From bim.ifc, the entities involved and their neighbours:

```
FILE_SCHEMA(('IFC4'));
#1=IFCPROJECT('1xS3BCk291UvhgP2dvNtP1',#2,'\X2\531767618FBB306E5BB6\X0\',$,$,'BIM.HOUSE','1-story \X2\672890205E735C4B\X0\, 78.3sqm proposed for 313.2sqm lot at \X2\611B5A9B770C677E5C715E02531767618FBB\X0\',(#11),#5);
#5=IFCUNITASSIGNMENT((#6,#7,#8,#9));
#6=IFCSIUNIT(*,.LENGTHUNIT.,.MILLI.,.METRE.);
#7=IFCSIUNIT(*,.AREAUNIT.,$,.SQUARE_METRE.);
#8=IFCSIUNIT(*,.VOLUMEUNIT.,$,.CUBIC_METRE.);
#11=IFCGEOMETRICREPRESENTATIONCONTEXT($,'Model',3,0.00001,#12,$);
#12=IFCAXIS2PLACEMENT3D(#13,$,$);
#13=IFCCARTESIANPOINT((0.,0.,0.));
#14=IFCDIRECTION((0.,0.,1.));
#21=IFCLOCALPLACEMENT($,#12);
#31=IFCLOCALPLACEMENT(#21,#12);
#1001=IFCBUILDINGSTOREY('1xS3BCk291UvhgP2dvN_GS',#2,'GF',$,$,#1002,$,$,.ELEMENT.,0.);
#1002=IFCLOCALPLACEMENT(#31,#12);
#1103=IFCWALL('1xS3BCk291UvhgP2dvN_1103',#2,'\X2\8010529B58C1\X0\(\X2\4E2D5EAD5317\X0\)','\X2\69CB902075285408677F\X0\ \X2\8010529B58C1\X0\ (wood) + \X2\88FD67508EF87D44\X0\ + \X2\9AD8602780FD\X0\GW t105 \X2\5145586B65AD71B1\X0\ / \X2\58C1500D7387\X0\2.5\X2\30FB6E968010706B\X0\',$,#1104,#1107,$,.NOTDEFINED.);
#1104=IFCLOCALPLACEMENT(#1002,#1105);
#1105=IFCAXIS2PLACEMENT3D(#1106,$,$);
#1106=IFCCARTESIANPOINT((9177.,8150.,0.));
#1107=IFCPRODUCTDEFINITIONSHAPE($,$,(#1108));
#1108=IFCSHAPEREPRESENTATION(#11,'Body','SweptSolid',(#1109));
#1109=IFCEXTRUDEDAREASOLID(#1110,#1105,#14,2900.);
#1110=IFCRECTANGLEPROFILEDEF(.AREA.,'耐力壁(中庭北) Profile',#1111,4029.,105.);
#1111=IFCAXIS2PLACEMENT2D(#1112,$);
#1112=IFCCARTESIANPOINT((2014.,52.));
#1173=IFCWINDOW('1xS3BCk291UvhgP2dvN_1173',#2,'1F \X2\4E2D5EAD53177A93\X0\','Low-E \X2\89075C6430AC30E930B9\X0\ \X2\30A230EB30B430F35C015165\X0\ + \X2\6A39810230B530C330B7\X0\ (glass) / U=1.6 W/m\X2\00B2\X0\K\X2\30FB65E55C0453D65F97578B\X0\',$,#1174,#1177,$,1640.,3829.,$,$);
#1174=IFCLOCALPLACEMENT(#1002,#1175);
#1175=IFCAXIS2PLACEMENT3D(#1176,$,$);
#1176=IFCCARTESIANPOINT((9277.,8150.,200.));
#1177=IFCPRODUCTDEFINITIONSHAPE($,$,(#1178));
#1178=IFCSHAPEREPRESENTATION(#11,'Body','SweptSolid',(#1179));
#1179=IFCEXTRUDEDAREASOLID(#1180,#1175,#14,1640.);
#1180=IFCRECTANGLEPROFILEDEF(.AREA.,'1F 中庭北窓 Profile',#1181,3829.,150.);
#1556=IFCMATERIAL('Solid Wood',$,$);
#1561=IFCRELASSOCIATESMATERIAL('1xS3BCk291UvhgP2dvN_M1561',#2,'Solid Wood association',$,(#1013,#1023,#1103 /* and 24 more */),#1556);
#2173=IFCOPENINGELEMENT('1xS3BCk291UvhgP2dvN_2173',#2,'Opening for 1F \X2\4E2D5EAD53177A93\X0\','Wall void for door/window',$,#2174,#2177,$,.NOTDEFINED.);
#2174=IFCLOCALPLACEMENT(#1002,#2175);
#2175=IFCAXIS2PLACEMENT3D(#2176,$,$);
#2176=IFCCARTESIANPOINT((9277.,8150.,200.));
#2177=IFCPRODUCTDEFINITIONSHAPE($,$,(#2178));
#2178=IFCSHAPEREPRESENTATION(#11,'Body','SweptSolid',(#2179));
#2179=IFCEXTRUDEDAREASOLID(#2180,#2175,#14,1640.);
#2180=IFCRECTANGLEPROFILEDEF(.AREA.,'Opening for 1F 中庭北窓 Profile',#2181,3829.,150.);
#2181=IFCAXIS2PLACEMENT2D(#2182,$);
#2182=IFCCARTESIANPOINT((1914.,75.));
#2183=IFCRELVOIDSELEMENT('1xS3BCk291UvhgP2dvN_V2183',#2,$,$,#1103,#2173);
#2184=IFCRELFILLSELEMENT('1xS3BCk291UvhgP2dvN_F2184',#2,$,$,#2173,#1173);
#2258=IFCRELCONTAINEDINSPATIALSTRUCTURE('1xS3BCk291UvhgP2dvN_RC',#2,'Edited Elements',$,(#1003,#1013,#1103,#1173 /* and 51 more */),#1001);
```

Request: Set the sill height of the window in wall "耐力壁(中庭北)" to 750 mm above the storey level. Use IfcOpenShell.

```python
import numpy as np
import ifcopenshell
import ifcopenshell.api.geometry
import ifcopenshell.geom
import ifcopenshell.util.element
import ifcopenshell.util.placement
import ifcopenshell.util.shape
import ifcopenshell.util.unit

model = ifcopenshell.open("bim.ifc")
unit_scale = ifcopenshell.util.unit.calculate_unit_scale(model)

window = model.by_guid("1xS3BCk291UvhgP2dvN_1173")
opening = window.FillsVoids[0].RelatingOpeningElement
storey = ifcopenshell.util.element.get_container(window, ifc_class="IfcBuildingStorey")
level = ifcopenshell.util.placement.get_local_placement(storey.ObjectPlacement)[2, 3]

# The opening's origin need not be at the sill, so measure its lowest point.
shape = ifcopenshell.geom.create_shape(ifcopenshell.geom.settings(), opening)
bottom = ifcopenshell.util.shape.get_shape_bottom_elevation(shape, shape.geometry) / unit_scale
dz = level + 750.0 - bottom

shift = np.array([0.0, 0.0, dz])
# The window is not placed relative to its opening, so move both.
for product in (opening, window):
    matrix = ifcopenshell.util.placement.get_local_placement(product.ObjectPlacement)
    matrix[:3, 3] += shift
    ifcopenshell.api.geometry.edit_object_placement(model, product=product, matrix=matrix, is_si=False)

print(f"moved by {dz * unit_scale:+.3f} m")

model.write("bim_updated.ifc")
```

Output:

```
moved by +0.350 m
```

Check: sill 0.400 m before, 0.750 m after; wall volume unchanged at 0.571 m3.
